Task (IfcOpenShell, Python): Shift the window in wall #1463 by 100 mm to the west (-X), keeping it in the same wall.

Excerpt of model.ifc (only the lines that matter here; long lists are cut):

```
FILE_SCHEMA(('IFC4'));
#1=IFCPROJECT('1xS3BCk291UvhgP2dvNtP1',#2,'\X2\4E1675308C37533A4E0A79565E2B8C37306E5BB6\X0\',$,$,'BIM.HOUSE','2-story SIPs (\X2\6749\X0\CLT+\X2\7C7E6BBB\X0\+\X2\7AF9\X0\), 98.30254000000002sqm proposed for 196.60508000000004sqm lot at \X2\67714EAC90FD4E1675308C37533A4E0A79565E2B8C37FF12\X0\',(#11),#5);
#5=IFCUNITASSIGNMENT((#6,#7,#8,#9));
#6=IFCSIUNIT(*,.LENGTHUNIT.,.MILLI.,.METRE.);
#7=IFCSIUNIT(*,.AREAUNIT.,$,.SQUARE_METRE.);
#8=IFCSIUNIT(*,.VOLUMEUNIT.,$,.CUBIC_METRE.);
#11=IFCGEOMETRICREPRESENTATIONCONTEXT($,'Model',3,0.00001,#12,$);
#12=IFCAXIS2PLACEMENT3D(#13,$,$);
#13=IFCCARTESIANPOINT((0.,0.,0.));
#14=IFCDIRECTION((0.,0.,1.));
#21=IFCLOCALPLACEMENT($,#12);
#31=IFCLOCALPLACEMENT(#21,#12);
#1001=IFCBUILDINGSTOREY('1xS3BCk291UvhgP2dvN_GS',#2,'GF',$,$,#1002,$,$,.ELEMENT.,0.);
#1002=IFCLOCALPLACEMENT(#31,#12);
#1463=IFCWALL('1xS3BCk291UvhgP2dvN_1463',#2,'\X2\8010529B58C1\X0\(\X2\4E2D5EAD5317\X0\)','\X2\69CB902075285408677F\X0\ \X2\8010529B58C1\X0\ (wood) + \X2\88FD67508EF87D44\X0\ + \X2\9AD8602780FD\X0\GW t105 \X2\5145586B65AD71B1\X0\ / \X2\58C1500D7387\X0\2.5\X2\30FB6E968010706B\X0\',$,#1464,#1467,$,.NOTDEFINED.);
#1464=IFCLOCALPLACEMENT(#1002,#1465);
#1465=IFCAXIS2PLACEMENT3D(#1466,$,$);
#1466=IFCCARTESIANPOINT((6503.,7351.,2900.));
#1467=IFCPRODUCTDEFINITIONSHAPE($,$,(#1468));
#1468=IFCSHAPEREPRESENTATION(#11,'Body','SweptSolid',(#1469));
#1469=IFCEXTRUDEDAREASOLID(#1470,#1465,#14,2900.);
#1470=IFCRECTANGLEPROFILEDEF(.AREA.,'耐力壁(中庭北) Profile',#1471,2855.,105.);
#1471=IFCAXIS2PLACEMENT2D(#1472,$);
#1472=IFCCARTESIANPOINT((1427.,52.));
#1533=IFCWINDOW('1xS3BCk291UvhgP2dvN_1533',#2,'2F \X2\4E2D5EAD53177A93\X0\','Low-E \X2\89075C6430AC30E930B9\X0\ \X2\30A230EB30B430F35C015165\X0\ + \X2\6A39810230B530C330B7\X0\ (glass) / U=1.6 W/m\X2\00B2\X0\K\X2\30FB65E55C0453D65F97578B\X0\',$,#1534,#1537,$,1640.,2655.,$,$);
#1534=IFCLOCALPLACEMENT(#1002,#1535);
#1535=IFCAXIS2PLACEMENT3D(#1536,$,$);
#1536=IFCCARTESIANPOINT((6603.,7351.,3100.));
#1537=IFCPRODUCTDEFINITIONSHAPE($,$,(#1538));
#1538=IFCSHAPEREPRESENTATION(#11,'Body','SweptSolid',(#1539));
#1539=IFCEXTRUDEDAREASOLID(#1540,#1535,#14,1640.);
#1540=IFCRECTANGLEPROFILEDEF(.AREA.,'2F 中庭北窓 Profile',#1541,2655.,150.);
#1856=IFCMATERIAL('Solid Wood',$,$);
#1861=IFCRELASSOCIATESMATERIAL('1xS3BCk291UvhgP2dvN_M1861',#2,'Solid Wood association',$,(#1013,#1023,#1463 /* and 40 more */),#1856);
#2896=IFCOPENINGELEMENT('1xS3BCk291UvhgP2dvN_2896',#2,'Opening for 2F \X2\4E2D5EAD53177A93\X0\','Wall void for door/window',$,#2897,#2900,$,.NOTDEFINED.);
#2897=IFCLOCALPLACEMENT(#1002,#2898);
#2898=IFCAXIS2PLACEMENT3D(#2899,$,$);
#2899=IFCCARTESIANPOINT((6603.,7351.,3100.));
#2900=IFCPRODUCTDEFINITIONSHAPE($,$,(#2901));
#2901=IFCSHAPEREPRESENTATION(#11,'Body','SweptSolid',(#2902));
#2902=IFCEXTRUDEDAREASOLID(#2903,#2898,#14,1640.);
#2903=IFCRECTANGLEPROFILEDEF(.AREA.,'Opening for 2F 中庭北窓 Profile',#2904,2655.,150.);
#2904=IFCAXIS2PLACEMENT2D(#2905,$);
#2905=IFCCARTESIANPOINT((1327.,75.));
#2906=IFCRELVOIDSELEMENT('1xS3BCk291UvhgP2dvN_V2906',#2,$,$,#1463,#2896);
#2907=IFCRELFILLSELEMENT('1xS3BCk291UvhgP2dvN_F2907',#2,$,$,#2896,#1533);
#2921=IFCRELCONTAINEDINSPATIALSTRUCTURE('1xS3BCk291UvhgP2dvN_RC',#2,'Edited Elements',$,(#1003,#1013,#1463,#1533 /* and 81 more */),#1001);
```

```python
import ifcopenshell
import ifcopenshell.api.geometry
import ifcopenshell.util.placement
import ifcopenshell.util.unit

model = ifcopenshell.open("model.ifc")
unit_scale = ifcopenshell.util.unit.calculate_unit_scale(model)

window = model.by_id(1533)
opening = window.FillsVoids[0].RelatingOpeningElement
wall = opening.VoidsElements[0].RelatingBuildingElement

wall_matrix = ifcopenshell.util.placement.get_local_placement(wall.ObjectPlacement)
shift = wall_matrix[:3, 0] * -0.1 / unit_scale
before = ifcopenshell.util.placement.get_local_placement(window.ObjectPlacement)[:3, 3].copy()

# The window is not placed relative to its opening, so move both.
for product in (opening, window):
    matrix = ifcopenshell.util.placement.get_local_placement(product.ObjectPlacement)
    matrix[:3, 3] += shift
    ifcopenshell.api.geometry.edit_object_placement(model, product=product, matrix=matrix, is_si=False)

after = ifcopenshell.util.placement.get_local_placement(window.ObjectPlacement)[:3, 3]
print("window moved by", (after - before).round(3) + 0.0)

model.write("model_v2.ifc")
```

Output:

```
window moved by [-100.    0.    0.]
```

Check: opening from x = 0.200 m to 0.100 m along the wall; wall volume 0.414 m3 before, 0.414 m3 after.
